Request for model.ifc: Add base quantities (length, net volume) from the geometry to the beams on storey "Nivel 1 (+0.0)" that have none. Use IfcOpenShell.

First a look at what the model holds.

```python
import ifcopenshell
import ifcopenshell.util.element
import ifcopenshell.util.unit

model = ifcopenshell.open("model.ifc")
print(model.schema)
for unit_type in ("LENGTHUNIT", "AREAUNIT", "VOLUMEUNIT"):
    print(unit_type, ifcopenshell.util.unit.calculate_unit_scale(model, unit_type))
storey = next(s for s in model.by_type("IfcBuildingStorey") if s.Name == "Nivel 1 (+0.0)")
beams = [e for e in ifcopenshell.util.element.get_decomposition(storey) if e.is_a("IfcBeam")]
for e in sorted(beams, key=lambda e: e.id()):
    print(e.id(), e.is_a(), e.Name, list(ifcopenshell.util.element.get_psets(e, qtos_only=True)), sep=" | ")
```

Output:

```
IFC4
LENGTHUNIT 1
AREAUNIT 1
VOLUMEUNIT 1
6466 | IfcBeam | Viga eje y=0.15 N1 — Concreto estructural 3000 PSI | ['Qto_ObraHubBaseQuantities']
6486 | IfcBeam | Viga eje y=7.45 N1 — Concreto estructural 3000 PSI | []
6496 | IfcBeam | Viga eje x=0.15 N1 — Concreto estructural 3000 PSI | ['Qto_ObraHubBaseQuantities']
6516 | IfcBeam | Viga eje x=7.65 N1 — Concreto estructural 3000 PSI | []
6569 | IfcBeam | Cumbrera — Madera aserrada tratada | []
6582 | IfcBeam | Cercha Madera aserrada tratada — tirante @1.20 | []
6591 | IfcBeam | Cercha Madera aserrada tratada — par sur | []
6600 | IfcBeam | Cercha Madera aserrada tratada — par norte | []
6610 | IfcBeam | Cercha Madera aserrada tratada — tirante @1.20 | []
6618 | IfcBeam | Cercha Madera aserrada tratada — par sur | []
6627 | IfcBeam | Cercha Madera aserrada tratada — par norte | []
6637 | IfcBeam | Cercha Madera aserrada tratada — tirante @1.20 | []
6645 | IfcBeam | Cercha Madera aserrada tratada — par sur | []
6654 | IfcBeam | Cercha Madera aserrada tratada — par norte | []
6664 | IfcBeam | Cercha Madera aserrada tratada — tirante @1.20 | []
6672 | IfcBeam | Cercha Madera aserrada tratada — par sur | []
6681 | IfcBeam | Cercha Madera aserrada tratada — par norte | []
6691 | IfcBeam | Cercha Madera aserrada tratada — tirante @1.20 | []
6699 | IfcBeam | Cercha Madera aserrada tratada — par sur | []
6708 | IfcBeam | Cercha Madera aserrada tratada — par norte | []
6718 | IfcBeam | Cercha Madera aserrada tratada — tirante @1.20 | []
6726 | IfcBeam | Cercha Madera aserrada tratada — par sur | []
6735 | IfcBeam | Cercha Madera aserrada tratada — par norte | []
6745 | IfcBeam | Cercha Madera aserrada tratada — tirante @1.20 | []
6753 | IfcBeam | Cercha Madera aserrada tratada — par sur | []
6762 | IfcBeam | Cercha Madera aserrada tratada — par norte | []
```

```python
import ifcopenshell
import ifcopenshell.api.pset
import ifcopenshell.geom
import ifcopenshell.util.element
import ifcopenshell.util.shape
import ifcopenshell.util.unit

model = ifcopenshell.open("model.ifc")
unit_scale = ifcopenshell.util.unit.calculate_unit_scale(model)
volume_scale = ifcopenshell.util.unit.calculate_unit_scale(model, "VOLUMEUNIT")
settings = ifcopenshell.geom.settings()

storey = next(s for s in model.by_type("IfcBuildingStorey") if s.Name == "Nivel 1 (+0.0)")
beams = [e for e in ifcopenshell.util.element.get_decomposition(storey) if e.is_a("IfcBeam")]

for e in sorted(beams, key=lambda e: e.id()):
    if ifcopenshell.util.element.get_psets(e, qtos_only=True, should_inherit=False):
        continue
    # Geometry comes back in metres, in the element's own axes.
    shape = ifcopenshell.geom.create_shape(settings, e)
    values = {
        "Length": ifcopenshell.util.shape.get_max_xyz(shape.geometry) / unit_scale,
        "NetVolume": ifcopenshell.util.shape.get_volume(shape.geometry) / volume_scale,
    }
    qto = ifcopenshell.api.pset.add_qto(model, product=e, name="Qto_BeamBaseQuantities")
    ifcopenshell.api.pset.edit_qto(model, qto=qto, properties=values)
    print(e.id(), {k: round(v, 3) for k, v in values.items()})

model.write("model_v2.ifc")
```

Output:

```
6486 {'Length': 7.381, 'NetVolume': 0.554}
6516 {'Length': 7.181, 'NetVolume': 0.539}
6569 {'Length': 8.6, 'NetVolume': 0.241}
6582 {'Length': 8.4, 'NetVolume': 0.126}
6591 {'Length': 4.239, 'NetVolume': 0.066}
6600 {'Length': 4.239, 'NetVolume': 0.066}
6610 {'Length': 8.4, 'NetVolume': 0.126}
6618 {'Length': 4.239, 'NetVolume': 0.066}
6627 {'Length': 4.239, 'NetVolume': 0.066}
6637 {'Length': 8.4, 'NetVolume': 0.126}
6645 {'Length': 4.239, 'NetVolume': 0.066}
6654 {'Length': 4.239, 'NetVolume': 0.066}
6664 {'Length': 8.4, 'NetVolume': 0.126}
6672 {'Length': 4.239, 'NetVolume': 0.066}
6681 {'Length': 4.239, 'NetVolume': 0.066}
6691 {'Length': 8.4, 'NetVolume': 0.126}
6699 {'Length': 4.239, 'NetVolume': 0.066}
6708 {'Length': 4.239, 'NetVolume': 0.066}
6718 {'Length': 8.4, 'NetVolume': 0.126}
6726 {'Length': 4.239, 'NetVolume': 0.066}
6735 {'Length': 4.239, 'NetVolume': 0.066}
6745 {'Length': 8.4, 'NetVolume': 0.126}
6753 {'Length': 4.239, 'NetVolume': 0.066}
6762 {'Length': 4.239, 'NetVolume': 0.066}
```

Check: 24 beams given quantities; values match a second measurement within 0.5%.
